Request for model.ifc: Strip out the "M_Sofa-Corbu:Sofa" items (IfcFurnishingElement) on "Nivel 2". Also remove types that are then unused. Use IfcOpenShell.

First a look at what the model holds.

```python
import ifcopenshell
import ifcopenshell.util.element

model = ifcopenshell.open("model.ifc")
print(model.schema)
storey = next(s for s in model.by_type("IfcBuildingStorey") if s.Name == "Nivel 2")
furniture = [e for e in ifcopenshell.util.element.get_decomposition(storey) if e.is_a("IfcFurnishingElement")]
seen = {}
for e in furniture:
    element_type = ifcopenshell.util.element.get_type(e)
    name = element_type.Name if element_type not in (None, e) else None
    seen[name] = seen.get(name, 0) + 1
for name, count in sorted(seen.items(), key=str):
    print(count, "x", name)
```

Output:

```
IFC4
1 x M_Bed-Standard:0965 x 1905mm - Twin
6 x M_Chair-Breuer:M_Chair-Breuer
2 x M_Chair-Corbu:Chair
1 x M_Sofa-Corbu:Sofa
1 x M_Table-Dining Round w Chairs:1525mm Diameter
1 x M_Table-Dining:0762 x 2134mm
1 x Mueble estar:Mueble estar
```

```python
import ifcopenshell
import ifcopenshell.api.root
import ifcopenshell.util.element

model = ifcopenshell.open("model.ifc")

storey = next(s for s in model.by_type("IfcBuildingStorey") if s.Name == "Nivel 2")
furniture = [e for e in ifcopenshell.util.element.get_decomposition(storey) if e.is_a("IfcFurnishingElement")]
targets = [e for e in furniture if (t := ifcopenshell.util.element.get_type(e)) not in (None, e) and t.Name == "M_Sofa-Corbu:Sofa"]
types = {ifcopenshell.util.element.get_type(e) for e in targets} - {None, *targets}

for e in targets:
    ifcopenshell.api.root.remove_product(model, product=e)
print(len(targets), "removed")

unused = [t for t in types if not ifcopenshell.util.element.get_types(t)]
for t in unused:
    ifcopenshell.api.root.remove_product(model, product=t)
print(len(unused), "unused types removed")

model.write("model_updated.ifc")
```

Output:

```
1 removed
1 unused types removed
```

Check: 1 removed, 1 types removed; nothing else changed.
